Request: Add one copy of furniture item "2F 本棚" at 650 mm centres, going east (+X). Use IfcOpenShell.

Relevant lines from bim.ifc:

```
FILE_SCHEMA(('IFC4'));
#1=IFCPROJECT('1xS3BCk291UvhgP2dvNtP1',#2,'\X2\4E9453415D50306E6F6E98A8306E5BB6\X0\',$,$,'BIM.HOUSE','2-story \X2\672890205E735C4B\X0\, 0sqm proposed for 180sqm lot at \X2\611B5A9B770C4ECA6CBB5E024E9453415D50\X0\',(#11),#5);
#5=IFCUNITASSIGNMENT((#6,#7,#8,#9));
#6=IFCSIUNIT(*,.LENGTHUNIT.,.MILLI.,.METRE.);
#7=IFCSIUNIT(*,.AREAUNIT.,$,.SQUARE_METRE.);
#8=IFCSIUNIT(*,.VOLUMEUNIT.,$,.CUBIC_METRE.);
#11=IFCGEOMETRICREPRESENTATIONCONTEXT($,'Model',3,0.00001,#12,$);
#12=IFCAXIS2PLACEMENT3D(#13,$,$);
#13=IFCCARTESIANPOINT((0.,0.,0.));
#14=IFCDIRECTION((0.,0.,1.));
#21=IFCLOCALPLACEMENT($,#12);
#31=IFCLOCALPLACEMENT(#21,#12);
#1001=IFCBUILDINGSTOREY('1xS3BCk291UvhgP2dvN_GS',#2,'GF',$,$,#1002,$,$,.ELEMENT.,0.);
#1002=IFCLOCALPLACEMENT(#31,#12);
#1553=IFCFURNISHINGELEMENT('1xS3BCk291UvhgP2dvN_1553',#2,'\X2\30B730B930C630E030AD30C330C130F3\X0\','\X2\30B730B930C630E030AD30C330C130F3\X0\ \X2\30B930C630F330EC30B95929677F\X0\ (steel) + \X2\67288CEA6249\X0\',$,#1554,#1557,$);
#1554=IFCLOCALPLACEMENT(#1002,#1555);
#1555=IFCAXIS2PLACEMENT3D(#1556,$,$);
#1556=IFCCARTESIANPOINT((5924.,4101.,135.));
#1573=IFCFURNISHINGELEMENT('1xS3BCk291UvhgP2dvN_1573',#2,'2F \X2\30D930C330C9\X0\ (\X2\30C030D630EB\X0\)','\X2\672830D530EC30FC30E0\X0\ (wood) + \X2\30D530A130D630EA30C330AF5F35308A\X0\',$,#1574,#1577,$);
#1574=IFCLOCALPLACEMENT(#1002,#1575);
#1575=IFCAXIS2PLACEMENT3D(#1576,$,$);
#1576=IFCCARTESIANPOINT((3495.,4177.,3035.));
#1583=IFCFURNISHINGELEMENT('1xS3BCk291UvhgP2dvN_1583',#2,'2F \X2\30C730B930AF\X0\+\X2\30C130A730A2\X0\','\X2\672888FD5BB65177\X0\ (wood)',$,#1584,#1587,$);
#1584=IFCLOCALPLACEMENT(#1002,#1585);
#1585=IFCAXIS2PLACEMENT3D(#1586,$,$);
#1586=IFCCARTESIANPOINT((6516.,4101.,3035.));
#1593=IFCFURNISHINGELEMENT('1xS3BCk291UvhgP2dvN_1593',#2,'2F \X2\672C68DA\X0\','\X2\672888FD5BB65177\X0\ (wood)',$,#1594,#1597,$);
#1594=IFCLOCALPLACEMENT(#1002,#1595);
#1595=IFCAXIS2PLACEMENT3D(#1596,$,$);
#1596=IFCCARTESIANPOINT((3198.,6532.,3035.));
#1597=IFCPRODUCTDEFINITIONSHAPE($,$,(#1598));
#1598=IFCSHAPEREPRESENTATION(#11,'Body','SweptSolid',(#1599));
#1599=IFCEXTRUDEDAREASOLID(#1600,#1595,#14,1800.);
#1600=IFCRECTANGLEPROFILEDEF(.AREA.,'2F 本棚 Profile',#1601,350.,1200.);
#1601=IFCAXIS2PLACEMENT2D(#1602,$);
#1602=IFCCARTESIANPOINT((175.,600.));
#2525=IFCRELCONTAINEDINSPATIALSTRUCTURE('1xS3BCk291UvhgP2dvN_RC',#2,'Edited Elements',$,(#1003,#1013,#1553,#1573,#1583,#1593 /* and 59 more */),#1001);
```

```python
import numpy as np
import ifcopenshell
import ifcopenshell.api.geometry
import ifcopenshell.api.root
import ifcopenshell.util.element
import ifcopenshell.util.placement

model = ifcopenshell.open("bim.ifc")


def reuse_history(source, copy):
    """copy_class also copies each property set's owner history, people and application; keep the originals."""
    for rel in copy.IsDefinedBy:
        if rel.is_a("IfcRelDefinesByProperties") and (history := rel.RelatingPropertyDefinition.OwnerHistory):
            rel.RelatingPropertyDefinition.OwnerHistory = source.OwnerHistory
            ifcopenshell.util.element.remove_deep2(model, history)


source = model.by_guid("1xS3BCk291UvhgP2dvN_1593")
base = ifcopenshell.util.placement.get_local_placement(source.ObjectPlacement)
step = np.array([1.0, 0.0, 0.0]) * 650.0

for i in range(1, 2):
    copy = ifcopenshell.api.root.copy_class(model, product=source)
    copy.Representation = ifcopenshell.util.element.copy_deep(
        model, source.Representation, exclude=["IfcGeometricRepresentationContext", "IfcRepresentationMap"]
    )
    reuse_history(source, copy)
    matrix = base.copy()
    matrix[:3, 3] += i * step
    print("added at", matrix[:3, 3].round(3) + 0.0)
    ifcopenshell.api.geometry.edit_object_placement(model, product=copy, matrix=matrix, is_si=False)

model.write("bim_rev.ifc")
```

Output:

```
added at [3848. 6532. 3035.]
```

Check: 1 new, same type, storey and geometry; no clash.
